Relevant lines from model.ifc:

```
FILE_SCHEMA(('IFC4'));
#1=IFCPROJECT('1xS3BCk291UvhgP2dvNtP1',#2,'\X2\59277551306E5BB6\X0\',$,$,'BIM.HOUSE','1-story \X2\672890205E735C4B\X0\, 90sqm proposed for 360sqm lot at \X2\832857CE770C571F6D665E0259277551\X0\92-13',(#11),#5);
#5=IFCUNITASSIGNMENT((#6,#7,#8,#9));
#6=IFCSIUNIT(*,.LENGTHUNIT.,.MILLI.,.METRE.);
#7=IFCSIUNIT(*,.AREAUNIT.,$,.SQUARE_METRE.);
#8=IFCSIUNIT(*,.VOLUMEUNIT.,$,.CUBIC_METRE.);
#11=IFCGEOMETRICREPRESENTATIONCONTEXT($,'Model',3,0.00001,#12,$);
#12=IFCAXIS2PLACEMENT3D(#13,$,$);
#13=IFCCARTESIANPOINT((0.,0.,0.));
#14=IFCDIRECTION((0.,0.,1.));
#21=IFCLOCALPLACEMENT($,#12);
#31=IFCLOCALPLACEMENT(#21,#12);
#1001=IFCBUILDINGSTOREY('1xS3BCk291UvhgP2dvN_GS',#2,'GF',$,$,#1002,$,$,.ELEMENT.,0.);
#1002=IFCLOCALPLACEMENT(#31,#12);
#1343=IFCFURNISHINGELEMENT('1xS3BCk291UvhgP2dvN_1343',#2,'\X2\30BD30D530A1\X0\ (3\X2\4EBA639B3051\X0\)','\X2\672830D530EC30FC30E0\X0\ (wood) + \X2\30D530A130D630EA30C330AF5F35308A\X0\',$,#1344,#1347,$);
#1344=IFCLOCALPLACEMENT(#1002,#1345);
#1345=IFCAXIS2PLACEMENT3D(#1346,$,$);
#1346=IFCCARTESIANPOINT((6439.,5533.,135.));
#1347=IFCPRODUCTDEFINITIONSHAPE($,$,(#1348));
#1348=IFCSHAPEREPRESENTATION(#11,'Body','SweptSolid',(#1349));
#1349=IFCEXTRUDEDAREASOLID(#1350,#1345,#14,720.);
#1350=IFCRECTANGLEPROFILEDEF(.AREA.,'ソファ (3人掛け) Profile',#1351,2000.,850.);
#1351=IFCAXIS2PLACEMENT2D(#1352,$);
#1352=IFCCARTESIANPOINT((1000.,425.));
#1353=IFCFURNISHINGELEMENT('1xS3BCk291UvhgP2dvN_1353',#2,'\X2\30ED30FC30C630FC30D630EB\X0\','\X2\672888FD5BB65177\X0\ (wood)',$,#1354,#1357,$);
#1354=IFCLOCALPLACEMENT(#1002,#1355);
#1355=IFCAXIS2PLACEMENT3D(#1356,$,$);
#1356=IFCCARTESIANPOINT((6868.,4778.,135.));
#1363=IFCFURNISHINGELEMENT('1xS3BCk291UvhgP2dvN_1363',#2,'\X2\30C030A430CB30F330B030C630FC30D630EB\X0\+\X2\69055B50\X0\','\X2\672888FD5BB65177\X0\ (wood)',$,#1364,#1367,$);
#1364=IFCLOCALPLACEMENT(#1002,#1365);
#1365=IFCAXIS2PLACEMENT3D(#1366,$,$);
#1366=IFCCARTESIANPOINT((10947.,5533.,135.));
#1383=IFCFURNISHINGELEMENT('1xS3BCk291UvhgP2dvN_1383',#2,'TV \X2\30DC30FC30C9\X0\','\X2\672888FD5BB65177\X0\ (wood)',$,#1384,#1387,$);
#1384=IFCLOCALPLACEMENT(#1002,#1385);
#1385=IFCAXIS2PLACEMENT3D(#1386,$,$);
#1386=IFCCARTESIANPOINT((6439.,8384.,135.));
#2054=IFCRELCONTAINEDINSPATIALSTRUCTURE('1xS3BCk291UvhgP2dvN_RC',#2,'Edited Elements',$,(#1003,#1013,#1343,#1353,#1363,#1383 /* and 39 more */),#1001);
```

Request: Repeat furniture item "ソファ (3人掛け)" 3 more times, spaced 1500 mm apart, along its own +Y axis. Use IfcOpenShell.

```python
import ifcopenshell
import ifcopenshell.api.geometry
import ifcopenshell.api.root
import ifcopenshell.util.element
import ifcopenshell.util.placement

model = ifcopenshell.open("model.ifc")


def reuse_history(source, copy):
    """copy_class also copies each property set's owner history, people and application; keep the originals."""
    for rel in copy.IsDefinedBy:
        if rel.is_a("IfcRelDefinesByProperties") and (history := rel.RelatingPropertyDefinition.OwnerHistory):
            rel.RelatingPropertyDefinition.OwnerHistory = source.OwnerHistory
            ifcopenshell.util.element.remove_deep2(model, history)


source = model.by_id(1343)
base = ifcopenshell.util.placement.get_local_placement(source.ObjectPlacement)
step = base[:3, 1] * 1500.0

for i in range(1, 4):
    copy = ifcopenshell.api.root.copy_class(model, product=source)
    copy.Representation = ifcopenshell.util.element.copy_deep(
        model, source.Representation, exclude=["IfcGeometricRepresentationContext", "IfcRepresentationMap"]
    )
    reuse_history(source, copy)
    matrix = base.copy()
    matrix[:3, 3] += i * step
    print("added at", matrix[:3, 3].round(3) + 0.0)
    ifcopenshell.api.geometry.edit_object_placement(model, product=copy, matrix=matrix, is_si=False)

model.write("model_updated.ifc")
```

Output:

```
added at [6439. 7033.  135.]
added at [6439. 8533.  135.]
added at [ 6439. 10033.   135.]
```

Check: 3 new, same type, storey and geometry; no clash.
